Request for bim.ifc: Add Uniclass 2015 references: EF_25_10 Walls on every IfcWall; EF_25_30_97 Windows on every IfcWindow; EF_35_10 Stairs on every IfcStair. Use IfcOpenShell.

First a look at what the model holds.

```python
import ifcopenshell

model = ifcopenshell.open("bim.ifc")
print(model.schema)
print("classifications:", [c.Name for c in model.by_type("IfcClassification")])
for ifc_class in ("IfcDoor", "IfcRoof", "IfcStair", "IfcWall", "IfcWindow"):
    print(ifc_class, len(model.by_type(ifc_class)))
```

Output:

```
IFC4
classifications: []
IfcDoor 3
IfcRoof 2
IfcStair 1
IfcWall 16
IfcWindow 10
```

```python
import ifcopenshell
import ifcopenshell.api.classification

model = ifcopenshell.open("bim.ifc")

system = ifcopenshell.api.classification.add_classification(model, classification="Uniclass 2015")

codes = {
    "IfcWall": ("EF_25_10", "Walls"),
    "IfcWindow": ("EF_25_30_97", "Windows"),
    "IfcStair": ("EF_35_10", "Stairs"),
}
for ifc_class, (code, name) in codes.items():
    products = model.by_type(ifc_class)
    ifcopenshell.api.classification.add_reference(
        model, products=products, classification=system, identification=code, name=name
    )
    print(code, len(products))

model.write("bim_edited.ifc")
```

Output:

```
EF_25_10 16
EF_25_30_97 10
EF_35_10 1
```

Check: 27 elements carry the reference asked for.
